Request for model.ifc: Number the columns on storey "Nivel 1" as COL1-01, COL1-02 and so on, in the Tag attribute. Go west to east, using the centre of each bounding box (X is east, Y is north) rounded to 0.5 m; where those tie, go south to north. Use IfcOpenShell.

First a look at what the model holds.

```python
import ifcopenshell
import ifcopenshell.util.element
import ifcopenshell.util.placement

model = ifcopenshell.open("model.ifc")
print(model.schema)
storey = next(s for s in model.by_type("IfcBuildingStorey") if s.Name == "Nivel 1")
columns = [e for e in ifcopenshell.util.element.get_decomposition(storey) if e.is_a("IfcColumn")]
for e in sorted(columns, key=lambda e: e.id()):
    origin = ifcopenshell.util.placement.get_local_placement(e.ObjectPlacement)[:3, 3]
    print(e.id(), e.Tag, e.Name, origin.round(2) + 0.0, sep=" | ")
```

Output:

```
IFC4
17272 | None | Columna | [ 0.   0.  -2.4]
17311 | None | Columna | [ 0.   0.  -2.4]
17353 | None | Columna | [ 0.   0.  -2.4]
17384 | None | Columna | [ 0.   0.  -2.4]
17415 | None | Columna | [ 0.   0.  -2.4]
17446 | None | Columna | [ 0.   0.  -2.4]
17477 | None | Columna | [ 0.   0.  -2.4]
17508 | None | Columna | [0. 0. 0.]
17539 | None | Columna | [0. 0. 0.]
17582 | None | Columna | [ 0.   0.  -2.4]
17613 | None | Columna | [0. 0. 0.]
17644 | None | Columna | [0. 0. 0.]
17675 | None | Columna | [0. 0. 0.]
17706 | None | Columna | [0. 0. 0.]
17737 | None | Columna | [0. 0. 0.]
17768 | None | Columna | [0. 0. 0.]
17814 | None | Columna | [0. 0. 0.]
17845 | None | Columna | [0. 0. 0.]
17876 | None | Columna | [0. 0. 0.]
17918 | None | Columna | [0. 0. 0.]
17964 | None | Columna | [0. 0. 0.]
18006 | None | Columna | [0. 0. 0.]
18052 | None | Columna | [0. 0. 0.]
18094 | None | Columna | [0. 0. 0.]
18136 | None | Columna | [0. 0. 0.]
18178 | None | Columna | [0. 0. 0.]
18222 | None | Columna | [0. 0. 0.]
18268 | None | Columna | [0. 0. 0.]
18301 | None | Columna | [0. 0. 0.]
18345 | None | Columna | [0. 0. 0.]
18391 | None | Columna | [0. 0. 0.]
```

```python
import ifcopenshell
import ifcopenshell.geom
import ifcopenshell.util.element
import ifcopenshell.util.shape

model = ifcopenshell.open("model.ifc")
settings = ifcopenshell.geom.settings()
settings.set("use-world-coords", True)


def centre(element):
    shape = ifcopenshell.geom.create_shape(settings, element)
    return ifcopenshell.util.shape.get_bbox_centroid(shape.geometry)


storey = next(s for s in model.by_type("IfcBuildingStorey") if s.Name == "Nivel 1")
columns = [e for e in ifcopenshell.util.element.get_decomposition(storey) if e.is_a("IfcColumn")]

# Insertion points can sit at a corner or the storey origin, so sort by the geometry (in metres).
centres = {e: centre(e) for e in columns}
columns.sort(key=lambda e: (round(centres[e][0] / 0.5), centres[e][1]))

for i, e in enumerate(columns, start=1):
    number = f"COL1-{i:02d}"
    e.Tag = number
    print(e.id(), number)

model.write("model_rev.ifc")
```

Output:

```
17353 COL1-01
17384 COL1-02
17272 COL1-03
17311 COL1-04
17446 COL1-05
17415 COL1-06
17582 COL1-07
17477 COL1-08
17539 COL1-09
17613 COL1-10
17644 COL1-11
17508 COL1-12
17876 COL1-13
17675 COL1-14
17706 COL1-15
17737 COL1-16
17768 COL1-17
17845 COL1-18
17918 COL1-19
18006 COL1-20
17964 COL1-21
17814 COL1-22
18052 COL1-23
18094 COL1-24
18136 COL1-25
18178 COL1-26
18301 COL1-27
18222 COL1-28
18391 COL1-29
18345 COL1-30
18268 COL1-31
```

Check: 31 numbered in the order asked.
